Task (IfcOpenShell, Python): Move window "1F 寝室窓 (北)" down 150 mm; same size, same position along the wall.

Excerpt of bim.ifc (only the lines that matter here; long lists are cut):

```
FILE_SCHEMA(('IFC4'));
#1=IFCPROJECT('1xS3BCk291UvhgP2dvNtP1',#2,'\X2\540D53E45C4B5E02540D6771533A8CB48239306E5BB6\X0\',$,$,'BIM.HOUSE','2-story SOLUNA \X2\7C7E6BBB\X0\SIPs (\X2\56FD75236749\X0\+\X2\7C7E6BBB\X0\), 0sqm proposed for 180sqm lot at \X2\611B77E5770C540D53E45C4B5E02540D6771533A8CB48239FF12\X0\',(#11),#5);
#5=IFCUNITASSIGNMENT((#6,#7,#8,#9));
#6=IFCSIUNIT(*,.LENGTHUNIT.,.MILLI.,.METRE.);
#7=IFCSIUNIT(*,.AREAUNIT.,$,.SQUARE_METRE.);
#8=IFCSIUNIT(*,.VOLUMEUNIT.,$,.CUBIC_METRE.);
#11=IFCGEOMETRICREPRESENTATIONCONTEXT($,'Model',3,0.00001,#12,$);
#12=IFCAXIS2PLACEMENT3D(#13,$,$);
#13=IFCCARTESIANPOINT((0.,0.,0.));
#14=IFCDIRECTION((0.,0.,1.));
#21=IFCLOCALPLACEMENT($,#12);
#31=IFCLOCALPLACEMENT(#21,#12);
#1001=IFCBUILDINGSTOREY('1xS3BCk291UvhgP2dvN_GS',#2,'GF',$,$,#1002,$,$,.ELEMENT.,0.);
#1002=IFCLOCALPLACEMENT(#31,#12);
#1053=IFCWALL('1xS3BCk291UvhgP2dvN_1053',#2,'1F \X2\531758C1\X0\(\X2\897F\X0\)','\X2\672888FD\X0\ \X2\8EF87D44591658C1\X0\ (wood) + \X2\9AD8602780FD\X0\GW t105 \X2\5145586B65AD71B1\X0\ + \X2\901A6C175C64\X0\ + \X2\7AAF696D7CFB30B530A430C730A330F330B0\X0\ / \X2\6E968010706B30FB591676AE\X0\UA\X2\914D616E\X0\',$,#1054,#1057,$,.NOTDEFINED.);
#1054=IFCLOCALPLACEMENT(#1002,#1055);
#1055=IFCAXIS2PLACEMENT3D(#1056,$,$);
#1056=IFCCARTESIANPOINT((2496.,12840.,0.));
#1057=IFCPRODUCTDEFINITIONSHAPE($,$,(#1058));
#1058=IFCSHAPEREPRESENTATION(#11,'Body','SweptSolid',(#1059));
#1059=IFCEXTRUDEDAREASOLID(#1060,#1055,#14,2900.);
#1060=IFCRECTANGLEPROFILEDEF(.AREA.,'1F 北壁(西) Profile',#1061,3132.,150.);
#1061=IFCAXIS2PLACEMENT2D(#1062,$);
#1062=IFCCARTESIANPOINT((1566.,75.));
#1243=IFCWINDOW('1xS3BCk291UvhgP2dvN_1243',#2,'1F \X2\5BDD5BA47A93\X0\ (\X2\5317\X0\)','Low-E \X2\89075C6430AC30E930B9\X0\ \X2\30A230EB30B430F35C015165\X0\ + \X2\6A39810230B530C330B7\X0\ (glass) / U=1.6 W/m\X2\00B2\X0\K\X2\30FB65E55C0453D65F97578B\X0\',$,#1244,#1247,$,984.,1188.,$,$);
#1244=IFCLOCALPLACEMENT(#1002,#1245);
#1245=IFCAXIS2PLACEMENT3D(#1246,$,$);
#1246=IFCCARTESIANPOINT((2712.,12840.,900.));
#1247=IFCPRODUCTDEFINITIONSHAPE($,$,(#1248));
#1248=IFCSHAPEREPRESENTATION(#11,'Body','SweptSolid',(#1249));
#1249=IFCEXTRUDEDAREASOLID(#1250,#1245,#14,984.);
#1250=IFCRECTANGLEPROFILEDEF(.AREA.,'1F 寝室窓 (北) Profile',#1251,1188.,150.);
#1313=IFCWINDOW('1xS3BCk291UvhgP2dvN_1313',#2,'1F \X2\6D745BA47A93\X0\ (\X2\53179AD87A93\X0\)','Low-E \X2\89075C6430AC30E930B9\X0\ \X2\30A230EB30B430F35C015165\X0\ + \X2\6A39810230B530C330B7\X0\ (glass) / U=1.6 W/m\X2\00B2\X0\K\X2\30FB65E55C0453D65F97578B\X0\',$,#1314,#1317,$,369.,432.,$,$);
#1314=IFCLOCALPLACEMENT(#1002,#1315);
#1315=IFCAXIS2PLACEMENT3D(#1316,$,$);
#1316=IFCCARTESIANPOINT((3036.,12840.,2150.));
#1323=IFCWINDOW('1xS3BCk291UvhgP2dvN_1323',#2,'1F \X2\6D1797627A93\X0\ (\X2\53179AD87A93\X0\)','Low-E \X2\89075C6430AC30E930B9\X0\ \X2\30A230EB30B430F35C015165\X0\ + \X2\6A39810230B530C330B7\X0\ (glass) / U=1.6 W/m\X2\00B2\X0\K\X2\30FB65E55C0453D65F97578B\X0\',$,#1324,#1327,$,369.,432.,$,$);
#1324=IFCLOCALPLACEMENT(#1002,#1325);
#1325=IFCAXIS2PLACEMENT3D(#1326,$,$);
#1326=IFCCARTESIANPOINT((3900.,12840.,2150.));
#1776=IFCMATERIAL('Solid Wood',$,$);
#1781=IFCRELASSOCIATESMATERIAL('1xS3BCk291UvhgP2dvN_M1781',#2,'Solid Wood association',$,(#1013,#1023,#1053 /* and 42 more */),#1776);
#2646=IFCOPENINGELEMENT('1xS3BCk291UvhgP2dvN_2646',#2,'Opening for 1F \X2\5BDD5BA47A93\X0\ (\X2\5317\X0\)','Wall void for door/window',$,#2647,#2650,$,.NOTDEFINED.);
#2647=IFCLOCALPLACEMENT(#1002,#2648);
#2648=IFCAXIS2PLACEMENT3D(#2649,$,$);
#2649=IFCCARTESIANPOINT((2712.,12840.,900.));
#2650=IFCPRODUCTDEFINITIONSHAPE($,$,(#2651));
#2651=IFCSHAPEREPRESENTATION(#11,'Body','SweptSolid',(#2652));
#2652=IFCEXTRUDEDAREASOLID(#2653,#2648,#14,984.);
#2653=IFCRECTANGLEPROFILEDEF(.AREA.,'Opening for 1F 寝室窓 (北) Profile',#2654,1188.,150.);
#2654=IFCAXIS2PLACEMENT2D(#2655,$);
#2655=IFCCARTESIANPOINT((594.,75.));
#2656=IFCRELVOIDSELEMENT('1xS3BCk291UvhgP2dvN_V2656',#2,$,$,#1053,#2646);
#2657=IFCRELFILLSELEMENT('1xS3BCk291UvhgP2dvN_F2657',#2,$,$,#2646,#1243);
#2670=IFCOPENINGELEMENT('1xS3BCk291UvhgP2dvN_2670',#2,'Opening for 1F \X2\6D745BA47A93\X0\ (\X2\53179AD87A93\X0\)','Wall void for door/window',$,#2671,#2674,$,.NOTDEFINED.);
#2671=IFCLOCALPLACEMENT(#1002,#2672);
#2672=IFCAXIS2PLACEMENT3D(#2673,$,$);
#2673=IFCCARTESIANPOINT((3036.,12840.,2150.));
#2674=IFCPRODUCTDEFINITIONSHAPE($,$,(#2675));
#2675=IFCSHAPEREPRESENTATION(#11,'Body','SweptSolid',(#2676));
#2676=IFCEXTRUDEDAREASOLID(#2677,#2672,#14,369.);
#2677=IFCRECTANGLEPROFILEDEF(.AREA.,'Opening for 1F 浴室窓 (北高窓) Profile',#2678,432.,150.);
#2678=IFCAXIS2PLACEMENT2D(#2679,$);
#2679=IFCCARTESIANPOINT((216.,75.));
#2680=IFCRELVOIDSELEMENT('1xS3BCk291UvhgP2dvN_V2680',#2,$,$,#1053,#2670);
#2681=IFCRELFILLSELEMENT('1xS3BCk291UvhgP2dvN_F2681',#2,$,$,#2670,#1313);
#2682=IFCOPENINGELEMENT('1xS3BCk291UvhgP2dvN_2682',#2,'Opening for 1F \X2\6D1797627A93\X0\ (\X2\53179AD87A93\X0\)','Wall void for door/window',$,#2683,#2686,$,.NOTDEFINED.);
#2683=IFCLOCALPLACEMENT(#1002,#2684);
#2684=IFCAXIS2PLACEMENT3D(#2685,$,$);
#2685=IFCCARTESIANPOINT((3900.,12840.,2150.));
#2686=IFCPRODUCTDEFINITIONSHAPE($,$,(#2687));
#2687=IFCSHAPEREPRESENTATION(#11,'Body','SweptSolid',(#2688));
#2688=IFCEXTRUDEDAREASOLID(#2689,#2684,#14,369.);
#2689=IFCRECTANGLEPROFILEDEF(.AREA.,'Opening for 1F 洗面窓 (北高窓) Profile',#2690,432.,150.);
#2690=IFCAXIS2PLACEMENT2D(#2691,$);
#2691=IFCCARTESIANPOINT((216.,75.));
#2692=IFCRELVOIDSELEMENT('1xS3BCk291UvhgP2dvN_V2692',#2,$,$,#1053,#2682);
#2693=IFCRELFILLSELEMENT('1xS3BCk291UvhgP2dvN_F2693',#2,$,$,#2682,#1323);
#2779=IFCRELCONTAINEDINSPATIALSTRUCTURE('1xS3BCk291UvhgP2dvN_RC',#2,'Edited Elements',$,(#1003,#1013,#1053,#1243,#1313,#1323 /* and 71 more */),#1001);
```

```python
import numpy as np
import ifcopenshell
import ifcopenshell.api.geometry
import ifcopenshell.util.placement
import ifcopenshell.util.unit

model = ifcopenshell.open("bim.ifc")
unit_scale = ifcopenshell.util.unit.calculate_unit_scale(model)

window = model.by_id(1243)
opening = window.FillsVoids[0].RelatingOpeningElement
dz = -0.15 / unit_scale

shift = np.array([0.0, 0.0, dz])
# The window is not placed relative to its opening, so move both.
for product in (opening, window):
    matrix = ifcopenshell.util.placement.get_local_placement(product.ObjectPlacement)
    matrix[:3, 3] += shift
    ifcopenshell.api.geometry.edit_object_placement(model, product=product, matrix=matrix, is_si=False)

print(f"moved by {dz * unit_scale:+.3f} m")

model.write("bim_v2.ifc")
```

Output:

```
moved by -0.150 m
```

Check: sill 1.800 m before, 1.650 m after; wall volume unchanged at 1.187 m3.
